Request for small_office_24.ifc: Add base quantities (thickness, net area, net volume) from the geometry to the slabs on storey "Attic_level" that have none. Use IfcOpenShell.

First a look at what the model holds.

```python
import ifcopenshell
import ifcopenshell.util.element
import ifcopenshell.util.unit

model = ifcopenshell.open("small_office_24.ifc")
print(model.schema)
for unit_type in ("LENGTHUNIT", "AREAUNIT", "VOLUMEUNIT"):
    print(unit_type, ifcopenshell.util.unit.calculate_unit_scale(model, unit_type))
storey = next(s for s in model.by_type("IfcBuildingStorey") if s.Name == "Attic_level")
slabs = [e for e in ifcopenshell.util.element.get_decomposition(storey) if e.is_a("IfcSlab")]
for e in sorted(slabs, key=lambda e: e.id()):
    print(e.id(), e.is_a(), e.Name, list(ifcopenshell.util.element.get_psets(e, qtos_only=True)), sep=" | ")
```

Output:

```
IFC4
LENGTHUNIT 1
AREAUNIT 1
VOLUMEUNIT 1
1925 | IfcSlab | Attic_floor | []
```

```python
import ifcopenshell
import ifcopenshell.api.pset
import ifcopenshell.geom
import ifcopenshell.util.element
import ifcopenshell.util.shape
import ifcopenshell.util.unit

model = ifcopenshell.open("small_office_24.ifc")
unit_scale = ifcopenshell.util.unit.calculate_unit_scale(model)
area_scale = ifcopenshell.util.unit.calculate_unit_scale(model, "AREAUNIT")
volume_scale = ifcopenshell.util.unit.calculate_unit_scale(model, "VOLUMEUNIT")
settings = ifcopenshell.geom.settings()

storey = next(s for s in model.by_type("IfcBuildingStorey") if s.Name == "Attic_level")
slabs = [e for e in ifcopenshell.util.element.get_decomposition(storey) if e.is_a("IfcSlab")]

for e in sorted(slabs, key=lambda e: e.id()):
    if ifcopenshell.util.element.get_psets(e, qtos_only=True, should_inherit=False):
        continue
    # Geometry comes back in metres, in the element's own axes.
    shape = ifcopenshell.geom.create_shape(settings, e)
    values = {
        "Width": ifcopenshell.util.shape.get_z(shape.geometry) / unit_scale,
        "NetArea": ifcopenshell.util.shape.get_footprint_area(shape.geometry) / area_scale,
        "NetVolume": ifcopenshell.util.shape.get_volume(shape.geometry) / volume_scale,
    }
    qto = ifcopenshell.api.pset.add_qto(model, product=e, name="Qto_SlabBaseQuantities")
    ifcopenshell.api.pset.edit_qto(model, qto=qto, properties=values)
    print(e.id(), {k: round(v, 3) for k, v in values.items()})

model.write("small_office_24-out.ifc")
```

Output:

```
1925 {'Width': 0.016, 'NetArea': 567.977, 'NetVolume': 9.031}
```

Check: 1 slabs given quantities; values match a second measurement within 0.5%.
